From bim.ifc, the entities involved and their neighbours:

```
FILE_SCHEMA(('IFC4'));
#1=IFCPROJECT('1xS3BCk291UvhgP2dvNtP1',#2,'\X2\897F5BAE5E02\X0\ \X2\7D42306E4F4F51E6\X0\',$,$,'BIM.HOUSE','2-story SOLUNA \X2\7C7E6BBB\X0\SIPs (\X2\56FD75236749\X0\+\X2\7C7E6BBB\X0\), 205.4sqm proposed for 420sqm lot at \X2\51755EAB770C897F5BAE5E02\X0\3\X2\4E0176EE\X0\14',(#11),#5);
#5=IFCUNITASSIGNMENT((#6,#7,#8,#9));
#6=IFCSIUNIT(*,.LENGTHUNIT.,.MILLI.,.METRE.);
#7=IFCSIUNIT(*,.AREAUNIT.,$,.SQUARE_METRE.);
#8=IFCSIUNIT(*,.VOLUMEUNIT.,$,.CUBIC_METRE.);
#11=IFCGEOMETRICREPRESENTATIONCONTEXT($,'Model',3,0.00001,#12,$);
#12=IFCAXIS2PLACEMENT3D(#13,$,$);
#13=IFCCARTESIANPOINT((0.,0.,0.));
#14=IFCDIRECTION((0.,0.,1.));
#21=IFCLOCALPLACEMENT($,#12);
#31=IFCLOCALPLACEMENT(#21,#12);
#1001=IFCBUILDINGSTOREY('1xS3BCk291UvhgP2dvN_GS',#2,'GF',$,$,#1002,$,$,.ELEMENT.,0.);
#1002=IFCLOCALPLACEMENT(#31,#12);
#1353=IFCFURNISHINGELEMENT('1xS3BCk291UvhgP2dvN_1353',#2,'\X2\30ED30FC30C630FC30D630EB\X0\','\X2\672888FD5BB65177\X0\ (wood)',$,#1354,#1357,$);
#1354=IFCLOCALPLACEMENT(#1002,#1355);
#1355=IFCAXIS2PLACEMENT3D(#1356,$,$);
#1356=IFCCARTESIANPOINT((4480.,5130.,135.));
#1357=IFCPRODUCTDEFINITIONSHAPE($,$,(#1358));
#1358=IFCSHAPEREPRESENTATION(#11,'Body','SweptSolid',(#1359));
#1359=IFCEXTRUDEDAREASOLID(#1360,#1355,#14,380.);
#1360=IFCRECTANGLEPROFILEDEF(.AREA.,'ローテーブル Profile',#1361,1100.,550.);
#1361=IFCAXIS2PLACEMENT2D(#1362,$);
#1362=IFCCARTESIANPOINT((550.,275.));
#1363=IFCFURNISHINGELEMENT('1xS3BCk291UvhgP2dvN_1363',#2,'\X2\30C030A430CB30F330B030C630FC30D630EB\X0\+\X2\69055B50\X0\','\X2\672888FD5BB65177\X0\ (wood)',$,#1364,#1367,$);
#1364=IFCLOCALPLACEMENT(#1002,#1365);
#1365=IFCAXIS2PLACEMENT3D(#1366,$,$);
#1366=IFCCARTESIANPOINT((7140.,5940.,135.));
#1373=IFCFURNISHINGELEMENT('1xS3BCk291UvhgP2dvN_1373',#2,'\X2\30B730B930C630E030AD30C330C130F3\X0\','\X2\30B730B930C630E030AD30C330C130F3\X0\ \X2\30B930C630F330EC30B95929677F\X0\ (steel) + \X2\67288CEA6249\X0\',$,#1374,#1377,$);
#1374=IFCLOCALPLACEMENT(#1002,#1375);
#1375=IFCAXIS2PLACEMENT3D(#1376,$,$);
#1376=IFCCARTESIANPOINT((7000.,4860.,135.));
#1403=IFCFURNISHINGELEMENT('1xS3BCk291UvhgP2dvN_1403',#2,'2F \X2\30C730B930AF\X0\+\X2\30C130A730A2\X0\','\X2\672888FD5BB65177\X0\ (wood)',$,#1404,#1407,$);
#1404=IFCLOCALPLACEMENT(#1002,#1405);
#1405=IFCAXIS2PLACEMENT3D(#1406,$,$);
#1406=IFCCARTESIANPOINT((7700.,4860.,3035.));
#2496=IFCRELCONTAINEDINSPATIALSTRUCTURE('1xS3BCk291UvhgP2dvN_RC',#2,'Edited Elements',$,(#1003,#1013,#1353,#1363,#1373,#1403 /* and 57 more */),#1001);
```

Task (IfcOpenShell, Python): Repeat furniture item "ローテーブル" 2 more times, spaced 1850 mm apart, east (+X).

```python
import numpy as np
import ifcopenshell
import ifcopenshell.api.geometry
import ifcopenshell.api.root
import ifcopenshell.util.element
import ifcopenshell.util.placement

model = ifcopenshell.open("bim.ifc")


def reuse_history(source, copy):
    """copy_class also copies each property set's owner history, people and application; keep the originals."""
    for rel in copy.IsDefinedBy:
        if rel.is_a("IfcRelDefinesByProperties") and (history := rel.RelatingPropertyDefinition.OwnerHistory):
            rel.RelatingPropertyDefinition.OwnerHistory = source.OwnerHistory
            ifcopenshell.util.element.remove_deep2(model, history)


source = model.by_id(1353)
base = ifcopenshell.util.placement.get_local_placement(source.ObjectPlacement)
step = np.array([1.0, 0.0, 0.0]) * 1850.0

for i in range(1, 3):
    copy = ifcopenshell.api.root.copy_class(model, product=source)
    copy.Representation = ifcopenshell.util.element.copy_deep(
        model, source.Representation, exclude=["IfcGeometricRepresentationContext", "IfcRepresentationMap"]
    )
    reuse_history(source, copy)
    matrix = base.copy()
    matrix[:3, 3] += i * step
    print("added at", matrix[:3, 3].round(3) + 0.0)
    ifcopenshell.api.geometry.edit_object_placement(model, product=copy, matrix=matrix, is_si=False)

model.write("bim_updated.ifc")
```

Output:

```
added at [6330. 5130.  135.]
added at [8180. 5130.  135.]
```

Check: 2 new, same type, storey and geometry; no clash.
